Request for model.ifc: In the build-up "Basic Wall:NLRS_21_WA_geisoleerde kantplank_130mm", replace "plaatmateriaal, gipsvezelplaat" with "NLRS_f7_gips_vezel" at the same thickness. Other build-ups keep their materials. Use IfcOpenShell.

First a look at what the model holds.

```python
import ifcopenshell
import ifcopenshell.util.element

model = ifcopenshell.open("model.ifc")
print(model.schema)
for layer_set in model.by_type("IfcMaterialLayerSet"):
    if layer_set.LayerSetName == "Basic Wall:NLRS_21_WA_geisoleerde kantplank_130mm":
        for layer in layer_set.MaterialLayers:
            print(layer.id(), layer.Material and layer.Material.Name, layer.LayerThickness, sep=" | ")
        print(len(ifcopenshell.util.element.get_elements_by_material(model, layer_set)), "elements and types use it")
print(sorted(m.Name for m in model.by_type("IfcMaterial") if m.Name)[:60])
```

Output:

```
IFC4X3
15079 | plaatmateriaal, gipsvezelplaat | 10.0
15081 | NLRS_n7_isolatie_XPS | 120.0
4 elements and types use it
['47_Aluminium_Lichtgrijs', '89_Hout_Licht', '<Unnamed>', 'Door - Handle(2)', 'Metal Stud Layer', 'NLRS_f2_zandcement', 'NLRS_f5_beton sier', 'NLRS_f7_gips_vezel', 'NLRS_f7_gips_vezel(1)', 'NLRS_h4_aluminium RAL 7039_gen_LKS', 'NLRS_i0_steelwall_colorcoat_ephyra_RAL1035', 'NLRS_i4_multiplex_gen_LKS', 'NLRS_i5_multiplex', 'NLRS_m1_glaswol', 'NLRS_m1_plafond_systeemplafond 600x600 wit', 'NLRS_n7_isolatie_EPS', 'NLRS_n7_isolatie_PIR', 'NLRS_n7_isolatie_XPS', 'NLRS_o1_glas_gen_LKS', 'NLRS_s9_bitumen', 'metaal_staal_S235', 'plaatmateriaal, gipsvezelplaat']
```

```python
import ifcopenshell
import ifcopenshell.api.material

model = ifcopenshell.open("model.ifc")

layer_set = next(s for s in model.by_type("IfcMaterialLayerSet") if s.LayerSetName == "Basic Wall:NLRS_21_WA_geisoleerde kantplank_130mm")
layer = next(l for l in layer_set.MaterialLayers if l.Material and l.Material.Name == "plaatmateriaal, gipsvezelplaat")
material = next(m for m in model.by_type("IfcMaterial") if m.Name == "NLRS_f7_gips_vezel")

# Point this one layer at the other material; renaming the old one would change it everywhere.
ifcopenshell.api.material.edit_layer(model, layer=layer, attributes={"Name": material.Name}, material=material)

print([l.Material.Name if l.Material else None for l in layer_set.MaterialLayers])

model.write("model-out.ifc")
```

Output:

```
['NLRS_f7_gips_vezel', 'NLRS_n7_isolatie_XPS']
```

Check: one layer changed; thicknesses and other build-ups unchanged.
